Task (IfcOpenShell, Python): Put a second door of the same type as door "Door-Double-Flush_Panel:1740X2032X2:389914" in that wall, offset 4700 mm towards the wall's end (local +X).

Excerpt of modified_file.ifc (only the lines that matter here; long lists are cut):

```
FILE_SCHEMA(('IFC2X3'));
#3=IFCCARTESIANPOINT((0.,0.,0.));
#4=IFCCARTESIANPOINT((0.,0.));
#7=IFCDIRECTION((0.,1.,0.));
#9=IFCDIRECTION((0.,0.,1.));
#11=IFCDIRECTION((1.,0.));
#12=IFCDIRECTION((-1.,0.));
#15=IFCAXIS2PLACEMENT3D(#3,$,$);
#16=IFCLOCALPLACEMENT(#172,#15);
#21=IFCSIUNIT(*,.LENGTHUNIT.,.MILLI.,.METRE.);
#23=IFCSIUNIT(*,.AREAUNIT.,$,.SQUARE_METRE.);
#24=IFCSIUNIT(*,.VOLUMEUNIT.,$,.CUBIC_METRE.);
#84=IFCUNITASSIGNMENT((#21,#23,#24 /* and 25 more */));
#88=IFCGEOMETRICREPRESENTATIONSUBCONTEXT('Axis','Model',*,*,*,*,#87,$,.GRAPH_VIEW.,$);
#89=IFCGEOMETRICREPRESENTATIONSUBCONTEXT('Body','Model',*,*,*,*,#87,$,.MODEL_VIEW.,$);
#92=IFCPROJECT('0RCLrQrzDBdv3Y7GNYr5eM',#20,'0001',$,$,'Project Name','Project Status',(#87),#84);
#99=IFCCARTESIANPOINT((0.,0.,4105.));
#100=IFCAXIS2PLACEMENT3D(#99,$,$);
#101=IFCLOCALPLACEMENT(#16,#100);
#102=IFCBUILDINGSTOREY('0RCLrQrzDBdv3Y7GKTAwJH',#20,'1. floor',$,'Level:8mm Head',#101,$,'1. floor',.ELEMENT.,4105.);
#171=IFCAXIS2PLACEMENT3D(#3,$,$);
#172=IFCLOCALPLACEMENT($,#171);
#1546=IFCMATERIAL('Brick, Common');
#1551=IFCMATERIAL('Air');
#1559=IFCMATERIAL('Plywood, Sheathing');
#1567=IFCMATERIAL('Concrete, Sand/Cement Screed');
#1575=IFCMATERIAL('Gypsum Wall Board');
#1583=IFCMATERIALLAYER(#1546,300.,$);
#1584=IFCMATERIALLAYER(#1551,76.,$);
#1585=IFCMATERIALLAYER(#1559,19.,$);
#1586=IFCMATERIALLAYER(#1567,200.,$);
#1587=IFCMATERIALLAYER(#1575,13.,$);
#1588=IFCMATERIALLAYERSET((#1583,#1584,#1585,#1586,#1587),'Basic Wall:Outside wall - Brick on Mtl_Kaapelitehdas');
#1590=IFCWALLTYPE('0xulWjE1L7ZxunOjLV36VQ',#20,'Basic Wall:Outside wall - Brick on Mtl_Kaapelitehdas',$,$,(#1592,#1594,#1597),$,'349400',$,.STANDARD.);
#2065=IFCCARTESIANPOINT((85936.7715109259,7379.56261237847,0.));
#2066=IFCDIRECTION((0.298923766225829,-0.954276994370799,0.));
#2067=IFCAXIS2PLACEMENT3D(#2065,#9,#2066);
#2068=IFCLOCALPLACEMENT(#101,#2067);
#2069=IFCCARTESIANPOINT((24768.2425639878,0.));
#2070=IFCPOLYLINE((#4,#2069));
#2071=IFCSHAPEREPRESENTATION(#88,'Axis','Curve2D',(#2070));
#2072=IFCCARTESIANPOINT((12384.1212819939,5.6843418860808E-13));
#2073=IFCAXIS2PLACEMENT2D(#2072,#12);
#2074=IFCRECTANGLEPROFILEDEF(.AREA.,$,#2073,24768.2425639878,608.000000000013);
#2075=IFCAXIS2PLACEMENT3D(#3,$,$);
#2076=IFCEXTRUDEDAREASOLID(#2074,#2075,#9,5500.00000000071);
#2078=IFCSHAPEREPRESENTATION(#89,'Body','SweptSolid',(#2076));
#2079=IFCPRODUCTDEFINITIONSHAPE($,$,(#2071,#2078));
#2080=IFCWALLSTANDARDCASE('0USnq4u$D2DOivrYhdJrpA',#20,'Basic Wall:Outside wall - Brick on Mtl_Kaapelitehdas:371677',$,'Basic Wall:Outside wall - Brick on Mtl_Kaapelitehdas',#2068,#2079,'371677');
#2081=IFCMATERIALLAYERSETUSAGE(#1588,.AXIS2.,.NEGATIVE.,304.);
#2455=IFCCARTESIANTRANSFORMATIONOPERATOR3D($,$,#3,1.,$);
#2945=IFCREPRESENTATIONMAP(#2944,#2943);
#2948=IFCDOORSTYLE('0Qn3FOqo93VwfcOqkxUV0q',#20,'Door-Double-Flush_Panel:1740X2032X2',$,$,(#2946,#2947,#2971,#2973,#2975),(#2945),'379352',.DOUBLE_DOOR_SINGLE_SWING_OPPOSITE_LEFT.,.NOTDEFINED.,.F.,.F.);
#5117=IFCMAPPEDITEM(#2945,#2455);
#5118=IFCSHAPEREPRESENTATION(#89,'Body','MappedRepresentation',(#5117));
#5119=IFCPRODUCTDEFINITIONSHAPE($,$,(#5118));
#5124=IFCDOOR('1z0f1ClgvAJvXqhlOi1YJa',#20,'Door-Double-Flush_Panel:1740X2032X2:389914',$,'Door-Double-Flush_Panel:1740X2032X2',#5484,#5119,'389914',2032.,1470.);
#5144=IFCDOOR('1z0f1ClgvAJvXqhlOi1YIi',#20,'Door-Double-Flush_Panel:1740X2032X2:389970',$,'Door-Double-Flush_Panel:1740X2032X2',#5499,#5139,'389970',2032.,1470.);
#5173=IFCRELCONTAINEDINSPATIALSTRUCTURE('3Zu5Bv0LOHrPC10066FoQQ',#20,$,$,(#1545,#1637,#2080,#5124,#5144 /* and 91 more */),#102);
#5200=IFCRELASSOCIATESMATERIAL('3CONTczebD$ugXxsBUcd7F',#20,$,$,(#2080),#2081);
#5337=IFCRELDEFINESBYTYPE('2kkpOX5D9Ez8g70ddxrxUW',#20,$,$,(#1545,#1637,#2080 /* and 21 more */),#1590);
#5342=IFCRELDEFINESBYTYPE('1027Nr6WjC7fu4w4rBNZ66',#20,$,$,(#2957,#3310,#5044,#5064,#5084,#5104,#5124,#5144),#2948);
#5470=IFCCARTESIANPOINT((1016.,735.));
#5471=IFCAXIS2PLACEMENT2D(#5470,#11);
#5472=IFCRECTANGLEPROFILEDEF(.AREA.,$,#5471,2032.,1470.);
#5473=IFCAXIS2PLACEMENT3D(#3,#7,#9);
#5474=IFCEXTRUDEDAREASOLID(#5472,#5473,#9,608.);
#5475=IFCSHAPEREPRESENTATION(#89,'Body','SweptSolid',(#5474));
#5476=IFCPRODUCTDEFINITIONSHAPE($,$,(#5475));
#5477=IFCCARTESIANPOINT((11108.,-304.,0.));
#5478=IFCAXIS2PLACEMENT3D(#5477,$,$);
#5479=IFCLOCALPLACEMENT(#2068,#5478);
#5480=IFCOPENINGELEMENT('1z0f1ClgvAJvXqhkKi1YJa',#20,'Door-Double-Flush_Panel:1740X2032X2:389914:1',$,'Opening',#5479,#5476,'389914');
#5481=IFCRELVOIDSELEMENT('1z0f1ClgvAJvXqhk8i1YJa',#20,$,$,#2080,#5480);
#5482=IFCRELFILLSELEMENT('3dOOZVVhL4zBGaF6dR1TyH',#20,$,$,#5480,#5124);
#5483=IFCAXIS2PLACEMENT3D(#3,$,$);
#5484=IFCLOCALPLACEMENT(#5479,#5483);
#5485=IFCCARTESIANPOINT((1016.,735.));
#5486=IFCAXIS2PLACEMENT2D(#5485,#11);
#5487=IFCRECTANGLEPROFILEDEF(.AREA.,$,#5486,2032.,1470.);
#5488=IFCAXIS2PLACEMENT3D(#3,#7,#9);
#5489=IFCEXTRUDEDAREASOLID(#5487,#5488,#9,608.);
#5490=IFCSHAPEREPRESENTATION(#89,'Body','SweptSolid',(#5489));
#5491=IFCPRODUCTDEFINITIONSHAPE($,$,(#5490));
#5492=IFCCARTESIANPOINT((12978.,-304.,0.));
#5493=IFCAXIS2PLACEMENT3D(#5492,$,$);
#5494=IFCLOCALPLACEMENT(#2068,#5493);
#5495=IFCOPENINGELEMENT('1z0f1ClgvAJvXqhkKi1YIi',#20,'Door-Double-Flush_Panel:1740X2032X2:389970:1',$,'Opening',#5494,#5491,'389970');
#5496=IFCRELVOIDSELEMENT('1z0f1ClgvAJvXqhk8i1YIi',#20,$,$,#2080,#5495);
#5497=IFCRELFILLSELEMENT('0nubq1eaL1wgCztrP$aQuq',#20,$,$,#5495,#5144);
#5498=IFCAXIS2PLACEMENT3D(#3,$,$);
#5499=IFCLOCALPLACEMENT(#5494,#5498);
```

```python
import ifcopenshell
import ifcopenshell.api.feature
import ifcopenshell.api.geometry
import ifcopenshell.api.root
import ifcopenshell.geom
import ifcopenshell.util.element
import ifcopenshell.util.placement
import ifcopenshell.util.shape
import ifcopenshell.util.unit

model = ifcopenshell.open("modified_file.ifc")
unit_scale = ifcopenshell.util.unit.calculate_unit_scale(model)
settings = ifcopenshell.geom.settings()


def volume(element):
    """Net volume in cubic metres, openings subtracted."""
    shape = ifcopenshell.geom.create_shape(settings, element)
    return ifcopenshell.util.shape.get_volume(shape.geometry)


def reuse_history(source, copy):
    """copy_class also copies each property set's owner history, people and application; keep the originals."""
    for rel in copy.IsDefinedBy:
        if rel.is_a("IfcRelDefinesByProperties") and (history := rel.RelatingPropertyDefinition.OwnerHistory):
            rel.RelatingPropertyDefinition.OwnerHistory = source.OwnerHistory
            ifcopenshell.util.element.remove_deep2(model, history)


door = model.by_guid("1z0f1ClgvAJvXqhlOi1YJa")
opening = door.FillsVoids[0].RelatingOpeningElement
wall = opening.VoidsElements[0].RelatingBuildingElement
before = volume(wall)
shift = ifcopenshell.util.placement.get_local_placement(wall.ObjectPlacement)[:3, 0] * 4.7 / unit_scale

# copy_class copies the void relationship, type, container and properties, but no geometry.
new_opening = ifcopenshell.api.root.copy_class(model, product=opening)
new_opening.Representation = ifcopenshell.util.element.copy_deep(
    model, opening.Representation, exclude=["IfcGeometricRepresentationContext", "IfcRepresentationMap"]
)
new_opening.Name = "Door-Double-Flush_Panel:1740X2032X2"
new_opening.Tag = None
new_door = ifcopenshell.api.root.copy_class(model, product=door)
new_door.Representation = ifcopenshell.util.element.copy_deep(
    model, door.Representation, exclude=["IfcGeometricRepresentationContext", "IfcRepresentationMap"]
)
new_door.Name = "Door-Double-Flush_Panel:1740X2032X2"
new_door.Tag = None
reuse_history(door, new_door)
fills = ifcopenshell.api.feature.add_filling(model, opening=new_opening, element=new_door)
fills.OwnerHistory = new_door.OwnerHistory  # required in IFC2X3

for old, new in ((opening, new_opening), (door, new_door)):
    matrix = ifcopenshell.util.placement.get_local_placement(old.ObjectPlacement)
    matrix[:3, 3] += shift
    ifcopenshell.api.geometry.edit_object_placement(model, product=new, matrix=matrix, is_si=False)

after = volume(wall)

print(f"wall volume {before:.3f} -> {after:.3f} m3")

model.write("modified_file_updated.ifc")
```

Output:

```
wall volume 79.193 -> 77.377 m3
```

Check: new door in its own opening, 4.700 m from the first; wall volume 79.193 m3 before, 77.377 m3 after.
